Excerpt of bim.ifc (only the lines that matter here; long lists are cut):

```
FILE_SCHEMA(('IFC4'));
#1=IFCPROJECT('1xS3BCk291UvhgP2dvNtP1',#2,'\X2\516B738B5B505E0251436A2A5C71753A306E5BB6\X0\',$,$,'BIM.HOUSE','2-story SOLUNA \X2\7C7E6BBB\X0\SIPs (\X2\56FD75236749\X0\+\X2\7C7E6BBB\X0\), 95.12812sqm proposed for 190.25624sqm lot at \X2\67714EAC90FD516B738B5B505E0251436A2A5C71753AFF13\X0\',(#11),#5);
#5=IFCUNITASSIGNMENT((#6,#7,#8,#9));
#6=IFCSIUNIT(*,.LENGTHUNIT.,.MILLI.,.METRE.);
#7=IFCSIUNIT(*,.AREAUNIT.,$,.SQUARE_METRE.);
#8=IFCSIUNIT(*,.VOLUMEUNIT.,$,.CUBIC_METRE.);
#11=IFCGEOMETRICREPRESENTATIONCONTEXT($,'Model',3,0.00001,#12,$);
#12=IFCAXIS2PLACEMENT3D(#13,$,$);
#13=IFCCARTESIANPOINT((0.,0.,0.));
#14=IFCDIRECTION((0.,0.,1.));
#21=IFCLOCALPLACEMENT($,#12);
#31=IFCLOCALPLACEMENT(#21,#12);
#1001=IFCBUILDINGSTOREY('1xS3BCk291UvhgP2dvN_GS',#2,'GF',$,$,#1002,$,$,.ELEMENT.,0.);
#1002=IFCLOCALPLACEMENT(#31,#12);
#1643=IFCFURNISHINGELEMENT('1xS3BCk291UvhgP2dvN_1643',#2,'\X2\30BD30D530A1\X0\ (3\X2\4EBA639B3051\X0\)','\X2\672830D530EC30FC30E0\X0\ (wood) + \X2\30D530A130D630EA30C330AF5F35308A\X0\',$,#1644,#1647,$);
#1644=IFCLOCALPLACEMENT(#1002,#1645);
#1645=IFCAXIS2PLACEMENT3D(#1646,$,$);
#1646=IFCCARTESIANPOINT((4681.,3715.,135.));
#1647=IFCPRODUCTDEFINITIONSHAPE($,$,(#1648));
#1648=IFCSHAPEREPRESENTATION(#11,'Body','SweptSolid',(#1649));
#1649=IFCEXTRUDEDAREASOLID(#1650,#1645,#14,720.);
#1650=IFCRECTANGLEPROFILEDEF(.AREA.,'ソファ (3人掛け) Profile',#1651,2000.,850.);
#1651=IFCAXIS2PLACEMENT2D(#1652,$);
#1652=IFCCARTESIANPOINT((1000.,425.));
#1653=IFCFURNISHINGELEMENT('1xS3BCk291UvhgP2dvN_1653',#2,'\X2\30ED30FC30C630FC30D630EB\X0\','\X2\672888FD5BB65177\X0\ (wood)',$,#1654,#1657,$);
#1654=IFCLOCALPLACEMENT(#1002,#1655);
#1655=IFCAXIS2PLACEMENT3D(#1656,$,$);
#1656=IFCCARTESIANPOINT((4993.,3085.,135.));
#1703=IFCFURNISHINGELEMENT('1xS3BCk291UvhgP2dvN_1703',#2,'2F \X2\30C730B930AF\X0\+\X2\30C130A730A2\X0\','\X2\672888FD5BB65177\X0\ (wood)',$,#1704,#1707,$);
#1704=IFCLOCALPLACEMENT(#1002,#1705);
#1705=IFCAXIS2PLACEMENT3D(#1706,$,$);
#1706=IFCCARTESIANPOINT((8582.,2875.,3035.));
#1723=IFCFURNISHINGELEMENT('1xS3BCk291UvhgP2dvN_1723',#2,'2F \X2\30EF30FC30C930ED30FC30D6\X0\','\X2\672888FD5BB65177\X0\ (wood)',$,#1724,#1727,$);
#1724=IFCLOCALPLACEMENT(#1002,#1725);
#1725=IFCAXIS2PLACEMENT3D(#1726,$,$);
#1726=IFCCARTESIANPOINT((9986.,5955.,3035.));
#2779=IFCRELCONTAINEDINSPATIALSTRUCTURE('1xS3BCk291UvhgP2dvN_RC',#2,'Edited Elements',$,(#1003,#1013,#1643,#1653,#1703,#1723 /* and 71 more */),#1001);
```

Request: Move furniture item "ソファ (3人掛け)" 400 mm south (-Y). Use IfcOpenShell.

```python
import ifcopenshell
import ifcopenshell.api.geometry
import ifcopenshell.util.placement
import ifcopenshell.util.unit

model = ifcopenshell.open("bim.ifc")
unit_scale = ifcopenshell.util.unit.calculate_unit_scale(model)

item = model.by_guid("1xS3BCk291UvhgP2dvN_1643")
matrix = ifcopenshell.util.placement.get_local_placement(item.ObjectPlacement)
matrix[1, 3] -= 0.4 / unit_scale
ifcopenshell.api.geometry.edit_object_placement(model, product=item, matrix=matrix, is_si=False)

print(ifcopenshell.util.placement.get_local_placement(item.ObjectPlacement).round(3) + 0.0)

model.write("bim_rev.ifc")
```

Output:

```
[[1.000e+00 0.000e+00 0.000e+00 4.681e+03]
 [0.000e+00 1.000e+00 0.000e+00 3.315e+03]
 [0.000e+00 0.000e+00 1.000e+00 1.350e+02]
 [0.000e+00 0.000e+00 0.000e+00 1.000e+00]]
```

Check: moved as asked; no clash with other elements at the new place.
